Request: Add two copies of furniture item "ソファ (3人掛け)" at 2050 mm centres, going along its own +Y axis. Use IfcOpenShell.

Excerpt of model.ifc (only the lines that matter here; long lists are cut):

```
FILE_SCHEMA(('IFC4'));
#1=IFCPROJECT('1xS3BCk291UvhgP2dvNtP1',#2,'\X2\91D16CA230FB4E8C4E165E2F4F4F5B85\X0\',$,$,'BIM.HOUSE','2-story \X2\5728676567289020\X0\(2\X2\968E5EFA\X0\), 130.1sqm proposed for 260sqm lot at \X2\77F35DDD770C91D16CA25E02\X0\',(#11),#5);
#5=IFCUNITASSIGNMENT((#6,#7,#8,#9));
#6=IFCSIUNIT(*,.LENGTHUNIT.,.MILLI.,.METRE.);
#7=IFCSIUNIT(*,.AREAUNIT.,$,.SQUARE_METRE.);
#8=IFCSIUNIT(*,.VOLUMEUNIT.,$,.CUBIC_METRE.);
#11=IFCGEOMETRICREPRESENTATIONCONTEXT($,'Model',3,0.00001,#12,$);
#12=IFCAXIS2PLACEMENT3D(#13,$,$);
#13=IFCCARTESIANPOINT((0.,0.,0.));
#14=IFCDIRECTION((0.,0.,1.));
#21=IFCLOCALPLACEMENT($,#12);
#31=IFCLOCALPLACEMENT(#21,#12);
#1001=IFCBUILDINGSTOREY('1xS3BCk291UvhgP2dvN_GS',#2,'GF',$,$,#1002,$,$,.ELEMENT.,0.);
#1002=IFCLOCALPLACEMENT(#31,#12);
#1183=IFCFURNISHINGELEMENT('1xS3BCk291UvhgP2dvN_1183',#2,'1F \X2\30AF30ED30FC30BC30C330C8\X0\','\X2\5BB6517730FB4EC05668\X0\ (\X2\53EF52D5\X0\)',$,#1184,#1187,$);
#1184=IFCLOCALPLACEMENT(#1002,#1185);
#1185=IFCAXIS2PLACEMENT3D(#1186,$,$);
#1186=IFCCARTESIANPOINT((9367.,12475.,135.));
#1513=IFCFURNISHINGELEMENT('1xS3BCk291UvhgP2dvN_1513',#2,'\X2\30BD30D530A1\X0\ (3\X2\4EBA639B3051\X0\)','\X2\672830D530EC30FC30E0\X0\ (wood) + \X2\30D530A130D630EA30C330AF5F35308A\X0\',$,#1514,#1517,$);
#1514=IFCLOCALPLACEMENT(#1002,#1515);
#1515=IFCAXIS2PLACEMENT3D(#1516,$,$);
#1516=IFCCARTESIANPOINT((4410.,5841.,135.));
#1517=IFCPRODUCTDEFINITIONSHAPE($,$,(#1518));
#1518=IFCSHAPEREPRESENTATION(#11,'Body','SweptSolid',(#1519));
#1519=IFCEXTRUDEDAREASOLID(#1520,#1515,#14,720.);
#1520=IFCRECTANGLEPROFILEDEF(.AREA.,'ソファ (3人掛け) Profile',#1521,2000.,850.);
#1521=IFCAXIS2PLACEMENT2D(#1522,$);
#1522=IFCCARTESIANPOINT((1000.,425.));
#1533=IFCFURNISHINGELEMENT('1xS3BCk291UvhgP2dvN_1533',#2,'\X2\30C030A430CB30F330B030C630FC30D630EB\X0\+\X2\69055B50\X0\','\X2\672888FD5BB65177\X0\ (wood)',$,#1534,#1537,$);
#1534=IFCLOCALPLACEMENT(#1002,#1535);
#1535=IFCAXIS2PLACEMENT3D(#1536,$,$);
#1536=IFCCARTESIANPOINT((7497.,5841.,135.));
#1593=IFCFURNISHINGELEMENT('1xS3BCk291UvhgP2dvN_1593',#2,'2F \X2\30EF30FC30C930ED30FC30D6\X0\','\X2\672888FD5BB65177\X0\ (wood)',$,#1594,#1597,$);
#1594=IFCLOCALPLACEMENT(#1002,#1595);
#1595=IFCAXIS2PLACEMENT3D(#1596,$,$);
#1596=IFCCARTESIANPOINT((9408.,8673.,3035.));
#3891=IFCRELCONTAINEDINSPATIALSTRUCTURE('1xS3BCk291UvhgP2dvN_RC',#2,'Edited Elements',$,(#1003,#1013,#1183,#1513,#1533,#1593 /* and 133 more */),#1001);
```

```python
import ifcopenshell
import ifcopenshell.api.geometry
import ifcopenshell.api.root
import ifcopenshell.util.element
import ifcopenshell.util.placement

model = ifcopenshell.open("model.ifc")


def reuse_history(source, copy):
    """copy_class also copies each property set's owner history, people and application; keep the originals."""
    for rel in copy.IsDefinedBy:
        if rel.is_a("IfcRelDefinesByProperties") and (history := rel.RelatingPropertyDefinition.OwnerHistory):
            rel.RelatingPropertyDefinition.OwnerHistory = source.OwnerHistory
            ifcopenshell.util.element.remove_deep2(model, history)


source = model.by_guid("1xS3BCk291UvhgP2dvN_1513")
base = ifcopenshell.util.placement.get_local_placement(source.ObjectPlacement)
step = base[:3, 1] * 2050.0

for i in range(1, 3):
    copy = ifcopenshell.api.root.copy_class(model, product=source)
    copy.Representation = ifcopenshell.util.element.copy_deep(
        model, source.Representation, exclude=["IfcGeometricRepresentationContext", "IfcRepresentationMap"]
    )
    reuse_history(source, copy)
    matrix = base.copy()
    matrix[:3, 3] += i * step
    print("added at", matrix[:3, 3].round(3) + 0.0)
    ifcopenshell.api.geometry.edit_object_placement(model, product=copy, matrix=matrix, is_si=False)

model.write("model_rev.ifc")
```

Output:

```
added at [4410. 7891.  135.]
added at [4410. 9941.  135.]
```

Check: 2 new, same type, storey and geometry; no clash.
